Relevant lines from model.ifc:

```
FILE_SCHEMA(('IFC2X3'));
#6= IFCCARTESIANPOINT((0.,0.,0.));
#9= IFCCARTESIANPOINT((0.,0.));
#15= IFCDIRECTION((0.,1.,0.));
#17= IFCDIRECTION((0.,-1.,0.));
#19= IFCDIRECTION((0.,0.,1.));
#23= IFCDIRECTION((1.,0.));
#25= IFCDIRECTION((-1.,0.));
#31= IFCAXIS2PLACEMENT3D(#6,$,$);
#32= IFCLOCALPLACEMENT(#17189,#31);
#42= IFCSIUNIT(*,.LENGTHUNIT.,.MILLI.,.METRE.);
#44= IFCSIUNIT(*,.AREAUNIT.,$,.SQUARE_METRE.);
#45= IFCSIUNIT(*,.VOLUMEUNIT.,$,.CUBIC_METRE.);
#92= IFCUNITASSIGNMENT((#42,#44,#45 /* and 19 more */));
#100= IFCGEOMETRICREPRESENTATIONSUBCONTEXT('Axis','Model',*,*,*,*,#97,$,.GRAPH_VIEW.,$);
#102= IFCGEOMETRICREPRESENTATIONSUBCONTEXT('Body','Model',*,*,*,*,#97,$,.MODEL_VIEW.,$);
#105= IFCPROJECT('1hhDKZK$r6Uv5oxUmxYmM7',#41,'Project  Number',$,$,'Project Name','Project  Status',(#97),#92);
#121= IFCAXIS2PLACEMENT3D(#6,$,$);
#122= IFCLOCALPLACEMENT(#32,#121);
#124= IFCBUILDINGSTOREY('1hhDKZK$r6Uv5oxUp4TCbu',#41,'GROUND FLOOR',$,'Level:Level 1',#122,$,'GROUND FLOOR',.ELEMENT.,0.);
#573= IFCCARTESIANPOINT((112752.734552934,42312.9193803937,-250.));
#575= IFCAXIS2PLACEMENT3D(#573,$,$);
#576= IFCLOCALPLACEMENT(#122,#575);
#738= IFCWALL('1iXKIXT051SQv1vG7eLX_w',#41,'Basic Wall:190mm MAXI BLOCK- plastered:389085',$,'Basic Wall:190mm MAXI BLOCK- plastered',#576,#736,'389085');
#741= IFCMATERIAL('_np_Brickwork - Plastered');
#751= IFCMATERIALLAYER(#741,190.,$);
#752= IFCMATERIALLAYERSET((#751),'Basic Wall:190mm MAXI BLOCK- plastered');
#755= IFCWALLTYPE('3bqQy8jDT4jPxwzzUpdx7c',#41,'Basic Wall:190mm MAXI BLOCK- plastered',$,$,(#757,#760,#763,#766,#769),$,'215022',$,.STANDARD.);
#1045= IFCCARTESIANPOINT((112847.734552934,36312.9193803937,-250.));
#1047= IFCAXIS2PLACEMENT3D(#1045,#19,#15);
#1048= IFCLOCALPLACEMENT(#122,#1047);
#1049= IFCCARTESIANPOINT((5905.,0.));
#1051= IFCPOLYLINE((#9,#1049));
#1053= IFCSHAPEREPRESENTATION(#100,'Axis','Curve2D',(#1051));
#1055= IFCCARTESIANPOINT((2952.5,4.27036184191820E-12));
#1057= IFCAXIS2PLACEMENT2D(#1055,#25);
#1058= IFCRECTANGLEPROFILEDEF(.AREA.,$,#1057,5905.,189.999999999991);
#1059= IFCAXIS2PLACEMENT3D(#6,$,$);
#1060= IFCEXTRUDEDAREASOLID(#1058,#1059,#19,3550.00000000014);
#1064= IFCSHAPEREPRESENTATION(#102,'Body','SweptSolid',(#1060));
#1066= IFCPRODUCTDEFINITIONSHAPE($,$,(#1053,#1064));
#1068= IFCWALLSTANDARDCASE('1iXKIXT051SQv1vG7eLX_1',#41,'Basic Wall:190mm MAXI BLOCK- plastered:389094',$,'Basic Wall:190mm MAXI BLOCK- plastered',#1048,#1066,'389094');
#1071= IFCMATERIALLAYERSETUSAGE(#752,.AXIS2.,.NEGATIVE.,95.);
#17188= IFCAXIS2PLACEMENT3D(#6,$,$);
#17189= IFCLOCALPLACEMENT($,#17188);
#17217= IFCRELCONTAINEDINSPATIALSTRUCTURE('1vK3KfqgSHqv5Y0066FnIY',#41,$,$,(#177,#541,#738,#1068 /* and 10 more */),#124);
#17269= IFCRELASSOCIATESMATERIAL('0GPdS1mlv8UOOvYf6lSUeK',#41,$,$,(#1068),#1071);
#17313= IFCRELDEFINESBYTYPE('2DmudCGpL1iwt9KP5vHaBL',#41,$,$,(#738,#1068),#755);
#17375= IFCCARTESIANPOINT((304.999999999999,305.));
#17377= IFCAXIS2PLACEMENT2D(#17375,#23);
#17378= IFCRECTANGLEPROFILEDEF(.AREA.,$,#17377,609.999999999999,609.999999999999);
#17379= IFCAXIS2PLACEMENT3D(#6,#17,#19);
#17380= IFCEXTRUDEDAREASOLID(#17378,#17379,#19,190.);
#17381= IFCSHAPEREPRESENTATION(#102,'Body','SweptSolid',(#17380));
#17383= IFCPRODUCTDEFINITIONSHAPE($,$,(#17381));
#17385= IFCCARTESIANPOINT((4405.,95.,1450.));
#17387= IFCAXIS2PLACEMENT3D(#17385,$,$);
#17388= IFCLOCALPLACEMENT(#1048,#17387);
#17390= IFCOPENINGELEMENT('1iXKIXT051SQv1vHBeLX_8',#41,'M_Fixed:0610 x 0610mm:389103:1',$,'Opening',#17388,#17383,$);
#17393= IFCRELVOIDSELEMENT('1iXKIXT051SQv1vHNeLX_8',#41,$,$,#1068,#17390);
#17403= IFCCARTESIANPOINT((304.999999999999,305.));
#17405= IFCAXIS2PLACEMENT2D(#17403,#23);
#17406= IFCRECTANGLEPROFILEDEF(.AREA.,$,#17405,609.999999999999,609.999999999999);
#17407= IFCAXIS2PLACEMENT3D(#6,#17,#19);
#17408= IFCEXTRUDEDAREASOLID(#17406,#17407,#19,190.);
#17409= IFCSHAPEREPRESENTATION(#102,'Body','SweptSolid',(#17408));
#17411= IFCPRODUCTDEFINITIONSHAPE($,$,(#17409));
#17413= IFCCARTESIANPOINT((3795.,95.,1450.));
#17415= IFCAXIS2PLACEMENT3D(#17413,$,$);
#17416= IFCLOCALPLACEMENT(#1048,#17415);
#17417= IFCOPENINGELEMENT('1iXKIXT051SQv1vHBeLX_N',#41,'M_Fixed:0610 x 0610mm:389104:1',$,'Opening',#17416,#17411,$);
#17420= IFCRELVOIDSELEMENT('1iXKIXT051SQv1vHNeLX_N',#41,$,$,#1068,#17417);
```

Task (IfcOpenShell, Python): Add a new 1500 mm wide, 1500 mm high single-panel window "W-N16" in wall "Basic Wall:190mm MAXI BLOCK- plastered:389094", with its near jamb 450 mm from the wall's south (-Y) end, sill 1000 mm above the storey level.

```python
import numpy as np
import ifcopenshell
import ifcopenshell.api.feature
import ifcopenshell.api.geometry
import ifcopenshell.api.root
import ifcopenshell.api.spatial
import ifcopenshell.api.type
import ifcopenshell.geom
import ifcopenshell.util.element
import ifcopenshell.util.placement
import ifcopenshell.util.representation
import ifcopenshell.util.shape
import ifcopenshell.util.unit

model = ifcopenshell.open("model.ifc")
unit_scale = ifcopenshell.util.unit.calculate_unit_scale(model)
settings = ifcopenshell.geom.settings()


def volume(element):
    """Net volume in cubic metres, openings subtracted."""
    shape = ifcopenshell.geom.create_shape(settings, element)
    return ifcopenshell.util.shape.get_volume(shape.geometry)


wall = model.by_guid("1iXKIXT051SQv1vG7eLX_1")
storey = ifcopenshell.util.element.get_container(wall, ifc_class="IfcBuildingStorey")
context = ifcopenshell.util.representation.get_context(model, "Model", "Body", "MODEL_VIEW")
before = volume(wall)

width, height, from_end, sill = 1.5, 1.5, 0.45, 1  # metres

# The wall runs along its own X axis, and the end named is its -X end.
wall_shape = ifcopenshell.geom.create_shape(settings, wall)
x, y, z = ifcopenshell.util.shape.get_vertices(wall_shape.geometry).T
start = x.min() + from_end
face, thickness = float(y.min()), float(y.max() - y.min())
wall_matrix = ifcopenshell.util.placement.get_local_placement(wall.ObjectPlacement)
level = ifcopenshell.util.placement.get_local_placement(storey.ObjectPlacement)[2, 3]


def in_wall(x, y):
    """Placement at x, y metres in the wall's axes, at sill height."""
    matrix = wall_matrix.copy()
    matrix[:, 3] = wall_matrix @ np.array([x / unit_scale, y / unit_scale, 0.0, 1.0])
    matrix[2, 3] = level + sill / unit_scale
    return matrix


# Opening: a box that overshoots both wall faces by 50 mm.
opening = ifcopenshell.api.root.create_entity(model, ifc_class="IfcOpeningElement")
box = ifcopenshell.api.geometry.add_wall_representation(
    model, context=context, length=width, height=height, thickness=thickness + 0.1
)
ifcopenshell.api.geometry.assign_representation(model, product=opening, representation=box)
ifcopenshell.api.geometry.edit_object_placement(model, product=opening, matrix=in_wall(start, face - 0.05), is_si=False)
ifcopenshell.api.feature.add_feature(model, feature=opening, element=wall)

window = ifcopenshell.api.root.create_entity(model, ifc_class="IfcWindow", name="W-N16")
window.OverallWidth, window.OverallHeight = width / unit_scale, height / unit_scale
body = ifcopenshell.api.geometry.add_window_representation(
    model,
    context=context,
    overall_width=window.OverallWidth,
    overall_height=window.OverallHeight,
    partition_type="SINGLE_PANEL",
)
ifcopenshell.api.geometry.assign_representation(model, product=window, representation=body)
ifcopenshell.api.spatial.assign_container(model, products=[window], relating_structure=storey)
fills = ifcopenshell.api.feature.add_filling(model, opening=opening, element=window)
fills.OwnerHistory = window.OwnerHistory  # required in IFC2X3

# IFC2X3 keeps the operation on the window style.
style = ifcopenshell.api.root.create_entity(model, ifc_class="IfcWindowStyle", name="W-N16")
style.OperationType, style.ConstructionType = "SINGLE_PANEL", "NOTDEFINED"
style.ParameterTakesPrecedence = style.Sizeable = False
ifcopenshell.api.type.assign_type(model, related_objects=[window], relating_type=style)

# Centre the window in the wall's thickness.
ifcopenshell.api.geometry.edit_object_placement(model, product=window, matrix=in_wall(start, face), is_si=False)
window_shape = ifcopenshell.geom.create_shape(settings, window)
depth = ifcopenshell.util.shape.get_vertices(window_shape.geometry)[:, 1]
offset = face + thickness / 2 - (depth.min() + depth.max()) / 2
ifcopenshell.api.geometry.edit_object_placement(model, product=window, matrix=in_wall(start, offset), is_si=False)

after = volume(wall)

print(f"wall volume {before:.3f} -> {after:.3f} m3")

model.write("model_v2.ifc")
```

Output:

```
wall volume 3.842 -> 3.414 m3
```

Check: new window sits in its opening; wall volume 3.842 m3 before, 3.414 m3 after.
